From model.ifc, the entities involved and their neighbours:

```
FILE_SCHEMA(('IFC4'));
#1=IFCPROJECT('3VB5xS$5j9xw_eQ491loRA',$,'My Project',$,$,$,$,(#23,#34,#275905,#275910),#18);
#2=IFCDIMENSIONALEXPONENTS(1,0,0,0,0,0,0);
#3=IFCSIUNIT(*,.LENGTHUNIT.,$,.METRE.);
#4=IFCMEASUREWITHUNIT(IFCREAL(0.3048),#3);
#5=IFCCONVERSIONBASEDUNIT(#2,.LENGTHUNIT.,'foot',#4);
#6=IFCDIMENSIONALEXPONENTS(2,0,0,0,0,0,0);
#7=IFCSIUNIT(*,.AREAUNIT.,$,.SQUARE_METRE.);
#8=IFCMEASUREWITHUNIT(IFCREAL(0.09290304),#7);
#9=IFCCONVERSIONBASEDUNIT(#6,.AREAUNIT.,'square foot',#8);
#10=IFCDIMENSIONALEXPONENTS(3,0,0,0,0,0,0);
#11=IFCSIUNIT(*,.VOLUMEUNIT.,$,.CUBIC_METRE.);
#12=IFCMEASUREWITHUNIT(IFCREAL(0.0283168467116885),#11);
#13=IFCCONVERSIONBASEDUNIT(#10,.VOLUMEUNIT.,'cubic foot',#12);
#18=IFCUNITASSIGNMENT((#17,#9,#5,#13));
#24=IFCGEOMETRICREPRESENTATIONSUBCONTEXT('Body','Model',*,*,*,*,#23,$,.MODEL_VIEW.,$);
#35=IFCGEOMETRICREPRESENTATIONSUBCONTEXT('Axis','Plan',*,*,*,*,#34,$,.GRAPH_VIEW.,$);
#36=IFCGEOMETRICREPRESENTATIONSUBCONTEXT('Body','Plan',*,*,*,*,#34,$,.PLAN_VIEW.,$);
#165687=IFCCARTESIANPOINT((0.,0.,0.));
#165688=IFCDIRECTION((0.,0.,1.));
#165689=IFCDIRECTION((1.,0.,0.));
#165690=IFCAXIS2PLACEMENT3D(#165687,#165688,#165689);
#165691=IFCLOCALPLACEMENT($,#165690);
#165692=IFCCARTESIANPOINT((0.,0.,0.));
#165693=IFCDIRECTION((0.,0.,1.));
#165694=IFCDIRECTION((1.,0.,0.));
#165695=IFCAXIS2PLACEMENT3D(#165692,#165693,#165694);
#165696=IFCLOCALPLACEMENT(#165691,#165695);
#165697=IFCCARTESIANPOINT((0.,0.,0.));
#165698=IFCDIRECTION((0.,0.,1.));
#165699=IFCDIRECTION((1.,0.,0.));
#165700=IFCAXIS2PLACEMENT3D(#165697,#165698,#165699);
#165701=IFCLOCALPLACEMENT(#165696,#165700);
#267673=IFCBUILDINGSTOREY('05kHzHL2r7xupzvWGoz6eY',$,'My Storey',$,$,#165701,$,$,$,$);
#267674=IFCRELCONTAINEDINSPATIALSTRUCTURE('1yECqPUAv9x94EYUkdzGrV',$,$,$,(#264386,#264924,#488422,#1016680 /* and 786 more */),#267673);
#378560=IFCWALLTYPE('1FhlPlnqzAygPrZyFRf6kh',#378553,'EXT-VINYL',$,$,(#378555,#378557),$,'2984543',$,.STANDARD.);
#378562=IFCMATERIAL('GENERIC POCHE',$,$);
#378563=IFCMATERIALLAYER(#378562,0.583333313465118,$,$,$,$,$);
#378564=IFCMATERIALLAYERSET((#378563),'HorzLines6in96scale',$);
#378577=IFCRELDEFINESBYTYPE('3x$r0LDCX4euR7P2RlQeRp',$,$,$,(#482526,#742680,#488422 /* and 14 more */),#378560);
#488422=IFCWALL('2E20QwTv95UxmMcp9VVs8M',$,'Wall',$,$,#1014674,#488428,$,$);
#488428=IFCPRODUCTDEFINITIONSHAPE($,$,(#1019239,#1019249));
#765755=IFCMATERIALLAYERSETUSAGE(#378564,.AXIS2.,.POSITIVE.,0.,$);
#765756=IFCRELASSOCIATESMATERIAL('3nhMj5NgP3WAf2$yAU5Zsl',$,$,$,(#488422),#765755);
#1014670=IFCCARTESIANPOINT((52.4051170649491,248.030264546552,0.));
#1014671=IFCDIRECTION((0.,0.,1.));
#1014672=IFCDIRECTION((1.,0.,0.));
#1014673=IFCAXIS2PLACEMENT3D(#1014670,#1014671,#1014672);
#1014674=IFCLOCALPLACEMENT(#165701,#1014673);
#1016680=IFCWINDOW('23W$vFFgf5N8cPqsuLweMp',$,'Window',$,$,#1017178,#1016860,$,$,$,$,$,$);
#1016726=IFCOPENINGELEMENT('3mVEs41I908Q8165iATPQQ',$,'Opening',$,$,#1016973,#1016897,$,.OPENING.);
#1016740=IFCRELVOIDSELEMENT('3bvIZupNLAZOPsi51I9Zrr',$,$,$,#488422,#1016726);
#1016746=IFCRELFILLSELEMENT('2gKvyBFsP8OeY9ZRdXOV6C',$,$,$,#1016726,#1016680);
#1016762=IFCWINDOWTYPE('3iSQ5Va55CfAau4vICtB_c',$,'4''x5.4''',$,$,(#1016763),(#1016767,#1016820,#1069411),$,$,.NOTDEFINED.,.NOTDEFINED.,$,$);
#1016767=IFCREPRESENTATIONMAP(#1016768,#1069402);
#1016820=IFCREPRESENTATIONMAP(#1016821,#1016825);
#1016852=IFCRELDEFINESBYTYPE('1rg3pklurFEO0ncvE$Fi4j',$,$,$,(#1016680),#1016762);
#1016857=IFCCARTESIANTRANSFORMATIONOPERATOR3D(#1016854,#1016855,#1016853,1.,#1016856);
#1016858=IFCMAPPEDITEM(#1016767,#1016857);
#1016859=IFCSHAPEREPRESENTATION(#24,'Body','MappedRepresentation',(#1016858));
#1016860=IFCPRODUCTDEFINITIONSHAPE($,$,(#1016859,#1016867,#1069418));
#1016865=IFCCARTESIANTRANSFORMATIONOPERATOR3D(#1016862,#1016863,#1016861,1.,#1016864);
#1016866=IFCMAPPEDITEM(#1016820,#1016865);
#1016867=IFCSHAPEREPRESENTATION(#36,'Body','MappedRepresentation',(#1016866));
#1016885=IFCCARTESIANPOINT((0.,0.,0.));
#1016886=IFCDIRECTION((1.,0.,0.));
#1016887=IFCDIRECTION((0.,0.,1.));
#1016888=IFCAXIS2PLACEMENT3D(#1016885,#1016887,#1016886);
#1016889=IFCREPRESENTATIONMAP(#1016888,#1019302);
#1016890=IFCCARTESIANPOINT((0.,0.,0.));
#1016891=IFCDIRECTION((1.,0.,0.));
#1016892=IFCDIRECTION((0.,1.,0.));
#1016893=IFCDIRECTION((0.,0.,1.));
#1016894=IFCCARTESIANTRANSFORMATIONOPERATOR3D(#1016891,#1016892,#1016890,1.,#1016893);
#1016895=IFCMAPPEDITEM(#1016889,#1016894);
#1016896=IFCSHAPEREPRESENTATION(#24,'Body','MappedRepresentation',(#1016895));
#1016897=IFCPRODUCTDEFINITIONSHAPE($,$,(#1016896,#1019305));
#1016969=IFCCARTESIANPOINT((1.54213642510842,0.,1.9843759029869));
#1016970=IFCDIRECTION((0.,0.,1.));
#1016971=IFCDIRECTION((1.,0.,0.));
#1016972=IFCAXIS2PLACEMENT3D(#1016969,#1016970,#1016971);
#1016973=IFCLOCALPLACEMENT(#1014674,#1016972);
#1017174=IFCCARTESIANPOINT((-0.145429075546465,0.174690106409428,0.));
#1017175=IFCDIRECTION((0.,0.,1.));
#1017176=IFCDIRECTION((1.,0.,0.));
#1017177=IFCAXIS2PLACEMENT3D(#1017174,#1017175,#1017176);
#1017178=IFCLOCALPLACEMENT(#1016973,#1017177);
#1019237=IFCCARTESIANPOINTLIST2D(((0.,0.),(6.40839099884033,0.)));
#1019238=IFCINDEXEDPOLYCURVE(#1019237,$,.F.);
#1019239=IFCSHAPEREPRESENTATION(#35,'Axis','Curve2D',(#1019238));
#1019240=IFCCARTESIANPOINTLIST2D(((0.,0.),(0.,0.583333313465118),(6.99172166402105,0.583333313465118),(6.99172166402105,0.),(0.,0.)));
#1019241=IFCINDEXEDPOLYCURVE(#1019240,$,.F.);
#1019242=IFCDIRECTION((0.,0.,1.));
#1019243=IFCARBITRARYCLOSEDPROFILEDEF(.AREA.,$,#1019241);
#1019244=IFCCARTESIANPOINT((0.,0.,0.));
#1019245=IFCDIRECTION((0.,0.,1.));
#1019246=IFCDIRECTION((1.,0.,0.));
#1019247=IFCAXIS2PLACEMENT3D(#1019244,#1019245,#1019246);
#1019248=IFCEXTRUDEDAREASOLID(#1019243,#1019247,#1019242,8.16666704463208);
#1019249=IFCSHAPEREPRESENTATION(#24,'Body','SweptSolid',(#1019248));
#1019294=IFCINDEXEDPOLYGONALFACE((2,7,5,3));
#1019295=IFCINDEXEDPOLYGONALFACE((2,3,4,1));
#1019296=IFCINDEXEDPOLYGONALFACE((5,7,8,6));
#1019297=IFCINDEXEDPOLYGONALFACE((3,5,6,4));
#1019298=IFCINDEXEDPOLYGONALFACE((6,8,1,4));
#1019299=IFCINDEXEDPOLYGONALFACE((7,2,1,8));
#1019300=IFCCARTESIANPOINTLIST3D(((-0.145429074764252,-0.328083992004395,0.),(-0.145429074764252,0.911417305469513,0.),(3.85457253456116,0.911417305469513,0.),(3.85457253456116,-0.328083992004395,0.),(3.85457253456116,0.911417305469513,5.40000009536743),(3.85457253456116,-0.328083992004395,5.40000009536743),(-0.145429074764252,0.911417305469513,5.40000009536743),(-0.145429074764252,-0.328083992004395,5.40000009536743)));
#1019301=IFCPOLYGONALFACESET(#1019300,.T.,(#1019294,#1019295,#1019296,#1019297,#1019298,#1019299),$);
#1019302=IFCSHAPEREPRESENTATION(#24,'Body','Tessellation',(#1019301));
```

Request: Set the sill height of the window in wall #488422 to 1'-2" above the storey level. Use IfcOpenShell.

```python
import numpy as np
import ifcopenshell
import ifcopenshell.api.geometry
import ifcopenshell.geom
import ifcopenshell.util.element
import ifcopenshell.util.placement
import ifcopenshell.util.shape
import ifcopenshell.util.unit

model = ifcopenshell.open("model.ifc")
unit_scale = ifcopenshell.util.unit.calculate_unit_scale(model)

window = model.by_guid("23W$vFFgf5N8cPqsuLweMp")
opening = window.FillsVoids[0].RelatingOpeningElement
storey = ifcopenshell.util.element.get_container(window, ifc_class="IfcBuildingStorey")
level = ifcopenshell.util.placement.get_local_placement(storey.ObjectPlacement)[2, 3]

# The opening's origin need not be at the sill, so measure its lowest point.
shape = ifcopenshell.geom.create_shape(ifcopenshell.geom.settings(), opening)
bottom = ifcopenshell.util.shape.get_shape_bottom_elevation(shape, shape.geometry) / unit_scale
dz = level + 14 * 0.0254 / unit_scale - bottom

shift = np.array([0.0, 0.0, dz])
# The window is placed relative to its opening, so it follows when the opening moves.
matrix = ifcopenshell.util.placement.get_local_placement(opening.ObjectPlacement)
matrix[:3, 3] += shift
ifcopenshell.api.geometry.edit_object_placement(
    model, product=opening, matrix=matrix, is_si=False, should_transform_children=True
)

print(f"moved by {dz * unit_scale:+.3f} m")

model.write("model_edited.ifc")
```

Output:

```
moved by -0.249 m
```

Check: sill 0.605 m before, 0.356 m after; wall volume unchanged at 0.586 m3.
